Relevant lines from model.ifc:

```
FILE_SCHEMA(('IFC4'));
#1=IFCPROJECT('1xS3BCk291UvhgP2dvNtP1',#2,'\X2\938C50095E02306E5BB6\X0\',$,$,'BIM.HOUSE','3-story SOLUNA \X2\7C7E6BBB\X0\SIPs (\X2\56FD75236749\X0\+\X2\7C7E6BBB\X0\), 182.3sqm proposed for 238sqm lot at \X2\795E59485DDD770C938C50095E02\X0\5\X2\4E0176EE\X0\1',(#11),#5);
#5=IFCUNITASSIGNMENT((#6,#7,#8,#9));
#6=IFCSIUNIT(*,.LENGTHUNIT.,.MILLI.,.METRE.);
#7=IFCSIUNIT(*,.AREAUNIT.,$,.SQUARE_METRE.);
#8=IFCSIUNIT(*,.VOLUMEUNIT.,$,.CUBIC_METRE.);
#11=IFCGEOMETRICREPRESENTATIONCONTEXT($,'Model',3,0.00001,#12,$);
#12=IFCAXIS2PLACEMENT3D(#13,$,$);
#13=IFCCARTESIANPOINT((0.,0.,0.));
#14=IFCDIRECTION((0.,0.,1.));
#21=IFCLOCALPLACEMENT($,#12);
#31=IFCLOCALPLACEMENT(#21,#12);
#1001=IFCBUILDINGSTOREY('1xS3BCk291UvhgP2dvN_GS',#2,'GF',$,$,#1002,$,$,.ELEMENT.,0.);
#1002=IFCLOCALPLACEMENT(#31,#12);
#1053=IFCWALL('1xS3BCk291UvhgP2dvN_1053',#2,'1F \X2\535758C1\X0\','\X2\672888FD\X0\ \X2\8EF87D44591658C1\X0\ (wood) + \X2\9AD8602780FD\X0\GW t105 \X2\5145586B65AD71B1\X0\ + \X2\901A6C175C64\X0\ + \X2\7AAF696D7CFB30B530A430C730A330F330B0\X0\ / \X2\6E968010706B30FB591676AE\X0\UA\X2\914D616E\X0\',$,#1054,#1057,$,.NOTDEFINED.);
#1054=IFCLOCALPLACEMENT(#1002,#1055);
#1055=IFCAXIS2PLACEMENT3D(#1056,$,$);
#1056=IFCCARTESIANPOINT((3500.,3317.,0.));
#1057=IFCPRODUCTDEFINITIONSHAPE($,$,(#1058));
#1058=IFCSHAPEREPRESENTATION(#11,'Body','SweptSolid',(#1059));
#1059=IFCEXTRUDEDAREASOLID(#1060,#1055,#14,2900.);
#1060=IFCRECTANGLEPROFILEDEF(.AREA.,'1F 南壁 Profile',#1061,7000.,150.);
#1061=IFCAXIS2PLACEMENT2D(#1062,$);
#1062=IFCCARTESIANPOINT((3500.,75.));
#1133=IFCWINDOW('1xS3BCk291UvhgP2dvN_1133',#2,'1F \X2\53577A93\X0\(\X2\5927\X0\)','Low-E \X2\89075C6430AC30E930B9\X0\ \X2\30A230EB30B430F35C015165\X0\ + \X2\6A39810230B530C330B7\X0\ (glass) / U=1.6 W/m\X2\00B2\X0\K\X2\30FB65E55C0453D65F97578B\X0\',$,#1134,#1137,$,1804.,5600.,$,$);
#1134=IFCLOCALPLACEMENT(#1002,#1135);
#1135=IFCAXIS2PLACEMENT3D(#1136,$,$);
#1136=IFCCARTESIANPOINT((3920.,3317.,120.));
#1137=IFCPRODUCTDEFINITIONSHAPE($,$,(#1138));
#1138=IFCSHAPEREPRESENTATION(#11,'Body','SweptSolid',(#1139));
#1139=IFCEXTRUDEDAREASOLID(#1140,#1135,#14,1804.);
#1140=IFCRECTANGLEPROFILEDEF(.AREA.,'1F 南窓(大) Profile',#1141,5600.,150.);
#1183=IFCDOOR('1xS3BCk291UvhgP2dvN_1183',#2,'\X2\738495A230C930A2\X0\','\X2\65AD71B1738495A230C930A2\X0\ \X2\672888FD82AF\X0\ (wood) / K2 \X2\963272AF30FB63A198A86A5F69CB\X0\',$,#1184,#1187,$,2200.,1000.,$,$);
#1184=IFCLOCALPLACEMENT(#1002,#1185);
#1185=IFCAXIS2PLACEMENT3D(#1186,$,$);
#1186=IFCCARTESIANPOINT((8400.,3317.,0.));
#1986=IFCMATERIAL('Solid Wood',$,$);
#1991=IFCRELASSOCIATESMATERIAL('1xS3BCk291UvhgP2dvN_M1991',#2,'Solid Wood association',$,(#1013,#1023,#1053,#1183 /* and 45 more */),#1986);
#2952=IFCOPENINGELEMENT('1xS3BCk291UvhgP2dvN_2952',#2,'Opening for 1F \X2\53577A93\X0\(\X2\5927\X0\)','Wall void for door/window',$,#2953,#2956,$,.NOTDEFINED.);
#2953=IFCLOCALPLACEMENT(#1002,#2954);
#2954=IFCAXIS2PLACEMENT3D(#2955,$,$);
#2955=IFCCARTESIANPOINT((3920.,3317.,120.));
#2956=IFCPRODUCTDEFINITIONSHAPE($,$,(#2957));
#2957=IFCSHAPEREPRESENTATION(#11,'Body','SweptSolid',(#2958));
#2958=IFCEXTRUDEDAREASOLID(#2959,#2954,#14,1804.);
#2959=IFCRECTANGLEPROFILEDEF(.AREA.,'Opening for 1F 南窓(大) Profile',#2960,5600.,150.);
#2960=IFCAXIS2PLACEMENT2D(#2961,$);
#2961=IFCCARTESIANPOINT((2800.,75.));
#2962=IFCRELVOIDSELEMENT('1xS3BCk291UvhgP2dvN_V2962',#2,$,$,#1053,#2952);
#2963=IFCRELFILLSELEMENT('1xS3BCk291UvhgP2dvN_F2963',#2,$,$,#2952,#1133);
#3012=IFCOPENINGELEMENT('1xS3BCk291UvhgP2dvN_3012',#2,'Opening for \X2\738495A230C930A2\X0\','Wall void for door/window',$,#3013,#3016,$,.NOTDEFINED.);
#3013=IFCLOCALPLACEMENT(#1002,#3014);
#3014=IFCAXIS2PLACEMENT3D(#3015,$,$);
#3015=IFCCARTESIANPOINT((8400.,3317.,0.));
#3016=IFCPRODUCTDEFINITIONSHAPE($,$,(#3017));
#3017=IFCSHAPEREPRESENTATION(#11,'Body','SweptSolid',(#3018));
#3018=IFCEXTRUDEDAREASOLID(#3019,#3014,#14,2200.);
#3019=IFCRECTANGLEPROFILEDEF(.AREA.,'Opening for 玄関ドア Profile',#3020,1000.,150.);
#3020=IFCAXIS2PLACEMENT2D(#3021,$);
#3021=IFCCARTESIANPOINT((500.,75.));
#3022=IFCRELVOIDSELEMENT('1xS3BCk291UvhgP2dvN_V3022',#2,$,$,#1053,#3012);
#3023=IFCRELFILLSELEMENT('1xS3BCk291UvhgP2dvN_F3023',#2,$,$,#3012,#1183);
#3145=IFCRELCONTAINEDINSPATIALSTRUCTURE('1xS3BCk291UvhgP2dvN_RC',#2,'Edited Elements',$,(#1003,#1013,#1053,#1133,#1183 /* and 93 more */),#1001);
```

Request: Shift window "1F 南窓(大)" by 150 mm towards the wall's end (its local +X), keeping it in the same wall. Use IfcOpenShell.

```python
import ifcopenshell
import ifcopenshell.api.geometry
import ifcopenshell.util.placement
import ifcopenshell.util.unit

model = ifcopenshell.open("model.ifc")
unit_scale = ifcopenshell.util.unit.calculate_unit_scale(model)

window = model.by_guid("1xS3BCk291UvhgP2dvN_1133")
opening = window.FillsVoids[0].RelatingOpeningElement
wall = opening.VoidsElements[0].RelatingBuildingElement

wall_matrix = ifcopenshell.util.placement.get_local_placement(wall.ObjectPlacement)
shift = wall_matrix[:3, 0] * 0.15 / unit_scale
before = ifcopenshell.util.placement.get_local_placement(window.ObjectPlacement)[:3, 3].copy()

# The window is not placed relative to its opening, so move both.
for product in (opening, window):
    matrix = ifcopenshell.util.placement.get_local_placement(product.ObjectPlacement)
    matrix[:3, 3] += shift
    ifcopenshell.api.geometry.edit_object_placement(model, product=product, matrix=matrix, is_si=False)

after = ifcopenshell.util.placement.get_local_placement(window.ObjectPlacement)[:3, 3]
print("window moved by", (after - before).round(3) + 0.0)

model.write("model-out.ifc")
```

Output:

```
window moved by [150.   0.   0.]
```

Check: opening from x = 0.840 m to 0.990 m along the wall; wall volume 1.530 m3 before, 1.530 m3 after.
